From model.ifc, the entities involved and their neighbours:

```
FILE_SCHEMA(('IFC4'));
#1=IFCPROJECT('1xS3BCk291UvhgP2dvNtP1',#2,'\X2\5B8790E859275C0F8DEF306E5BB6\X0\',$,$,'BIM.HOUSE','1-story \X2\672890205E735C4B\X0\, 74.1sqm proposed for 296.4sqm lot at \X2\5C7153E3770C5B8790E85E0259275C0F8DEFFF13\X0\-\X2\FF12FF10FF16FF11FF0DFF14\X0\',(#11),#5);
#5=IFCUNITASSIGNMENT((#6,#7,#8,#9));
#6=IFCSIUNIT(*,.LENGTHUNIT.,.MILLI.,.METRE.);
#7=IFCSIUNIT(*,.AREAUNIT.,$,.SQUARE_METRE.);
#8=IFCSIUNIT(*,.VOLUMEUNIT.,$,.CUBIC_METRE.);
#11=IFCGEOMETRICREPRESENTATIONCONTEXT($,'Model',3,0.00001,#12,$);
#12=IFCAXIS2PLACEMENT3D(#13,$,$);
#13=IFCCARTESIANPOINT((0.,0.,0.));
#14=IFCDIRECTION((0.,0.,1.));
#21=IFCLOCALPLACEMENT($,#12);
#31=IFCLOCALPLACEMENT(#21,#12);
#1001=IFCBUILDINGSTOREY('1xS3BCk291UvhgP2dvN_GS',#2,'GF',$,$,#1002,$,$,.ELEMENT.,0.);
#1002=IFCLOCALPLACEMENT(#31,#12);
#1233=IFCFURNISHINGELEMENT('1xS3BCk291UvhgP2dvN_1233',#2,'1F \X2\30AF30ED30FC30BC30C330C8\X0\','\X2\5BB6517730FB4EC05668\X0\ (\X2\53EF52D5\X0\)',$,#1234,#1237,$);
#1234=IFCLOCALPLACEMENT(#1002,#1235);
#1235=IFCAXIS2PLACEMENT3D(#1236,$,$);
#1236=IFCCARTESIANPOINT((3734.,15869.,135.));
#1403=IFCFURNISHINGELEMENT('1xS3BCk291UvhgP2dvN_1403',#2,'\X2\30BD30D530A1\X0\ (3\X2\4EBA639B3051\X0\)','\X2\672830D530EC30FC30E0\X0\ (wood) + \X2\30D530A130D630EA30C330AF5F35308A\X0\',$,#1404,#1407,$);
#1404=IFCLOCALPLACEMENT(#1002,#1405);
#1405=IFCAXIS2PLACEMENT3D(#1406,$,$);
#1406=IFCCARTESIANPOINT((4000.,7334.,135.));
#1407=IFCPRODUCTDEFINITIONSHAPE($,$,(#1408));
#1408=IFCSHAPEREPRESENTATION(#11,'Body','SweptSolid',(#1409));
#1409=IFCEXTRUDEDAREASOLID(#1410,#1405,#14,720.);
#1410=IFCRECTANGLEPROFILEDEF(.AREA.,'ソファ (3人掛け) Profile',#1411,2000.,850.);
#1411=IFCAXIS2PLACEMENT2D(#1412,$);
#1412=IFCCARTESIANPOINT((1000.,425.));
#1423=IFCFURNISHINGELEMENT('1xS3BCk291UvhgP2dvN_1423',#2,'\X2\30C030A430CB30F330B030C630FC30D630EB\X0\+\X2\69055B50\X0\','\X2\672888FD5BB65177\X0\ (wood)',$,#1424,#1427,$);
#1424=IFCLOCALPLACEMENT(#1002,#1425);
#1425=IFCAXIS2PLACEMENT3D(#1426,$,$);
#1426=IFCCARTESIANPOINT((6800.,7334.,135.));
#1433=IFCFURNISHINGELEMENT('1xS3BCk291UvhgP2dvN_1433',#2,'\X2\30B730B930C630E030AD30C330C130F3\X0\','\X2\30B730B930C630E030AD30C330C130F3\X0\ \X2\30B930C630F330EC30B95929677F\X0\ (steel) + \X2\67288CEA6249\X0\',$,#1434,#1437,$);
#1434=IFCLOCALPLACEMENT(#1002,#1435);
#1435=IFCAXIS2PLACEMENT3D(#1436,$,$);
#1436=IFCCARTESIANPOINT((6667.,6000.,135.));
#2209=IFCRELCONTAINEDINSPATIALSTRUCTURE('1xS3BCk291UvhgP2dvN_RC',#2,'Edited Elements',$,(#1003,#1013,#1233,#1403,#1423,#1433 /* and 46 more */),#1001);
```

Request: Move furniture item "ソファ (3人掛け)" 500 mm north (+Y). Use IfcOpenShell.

```python
import ifcopenshell
import ifcopenshell.api.geometry
import ifcopenshell.util.placement
import ifcopenshell.util.unit

model = ifcopenshell.open("model.ifc")
unit_scale = ifcopenshell.util.unit.calculate_unit_scale(model)

item = model.by_guid("1xS3BCk291UvhgP2dvN_1403")
matrix = ifcopenshell.util.placement.get_local_placement(item.ObjectPlacement)
matrix[1, 3] += 0.5 / unit_scale
ifcopenshell.api.geometry.edit_object_placement(model, product=item, matrix=matrix, is_si=False)

print(ifcopenshell.util.placement.get_local_placement(item.ObjectPlacement).round(3) + 0.0)

model.write("model_edited.ifc")
```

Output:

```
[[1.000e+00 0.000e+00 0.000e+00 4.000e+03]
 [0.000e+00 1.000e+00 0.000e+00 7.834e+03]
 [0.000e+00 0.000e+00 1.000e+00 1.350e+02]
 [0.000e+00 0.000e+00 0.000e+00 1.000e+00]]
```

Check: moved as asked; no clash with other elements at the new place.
